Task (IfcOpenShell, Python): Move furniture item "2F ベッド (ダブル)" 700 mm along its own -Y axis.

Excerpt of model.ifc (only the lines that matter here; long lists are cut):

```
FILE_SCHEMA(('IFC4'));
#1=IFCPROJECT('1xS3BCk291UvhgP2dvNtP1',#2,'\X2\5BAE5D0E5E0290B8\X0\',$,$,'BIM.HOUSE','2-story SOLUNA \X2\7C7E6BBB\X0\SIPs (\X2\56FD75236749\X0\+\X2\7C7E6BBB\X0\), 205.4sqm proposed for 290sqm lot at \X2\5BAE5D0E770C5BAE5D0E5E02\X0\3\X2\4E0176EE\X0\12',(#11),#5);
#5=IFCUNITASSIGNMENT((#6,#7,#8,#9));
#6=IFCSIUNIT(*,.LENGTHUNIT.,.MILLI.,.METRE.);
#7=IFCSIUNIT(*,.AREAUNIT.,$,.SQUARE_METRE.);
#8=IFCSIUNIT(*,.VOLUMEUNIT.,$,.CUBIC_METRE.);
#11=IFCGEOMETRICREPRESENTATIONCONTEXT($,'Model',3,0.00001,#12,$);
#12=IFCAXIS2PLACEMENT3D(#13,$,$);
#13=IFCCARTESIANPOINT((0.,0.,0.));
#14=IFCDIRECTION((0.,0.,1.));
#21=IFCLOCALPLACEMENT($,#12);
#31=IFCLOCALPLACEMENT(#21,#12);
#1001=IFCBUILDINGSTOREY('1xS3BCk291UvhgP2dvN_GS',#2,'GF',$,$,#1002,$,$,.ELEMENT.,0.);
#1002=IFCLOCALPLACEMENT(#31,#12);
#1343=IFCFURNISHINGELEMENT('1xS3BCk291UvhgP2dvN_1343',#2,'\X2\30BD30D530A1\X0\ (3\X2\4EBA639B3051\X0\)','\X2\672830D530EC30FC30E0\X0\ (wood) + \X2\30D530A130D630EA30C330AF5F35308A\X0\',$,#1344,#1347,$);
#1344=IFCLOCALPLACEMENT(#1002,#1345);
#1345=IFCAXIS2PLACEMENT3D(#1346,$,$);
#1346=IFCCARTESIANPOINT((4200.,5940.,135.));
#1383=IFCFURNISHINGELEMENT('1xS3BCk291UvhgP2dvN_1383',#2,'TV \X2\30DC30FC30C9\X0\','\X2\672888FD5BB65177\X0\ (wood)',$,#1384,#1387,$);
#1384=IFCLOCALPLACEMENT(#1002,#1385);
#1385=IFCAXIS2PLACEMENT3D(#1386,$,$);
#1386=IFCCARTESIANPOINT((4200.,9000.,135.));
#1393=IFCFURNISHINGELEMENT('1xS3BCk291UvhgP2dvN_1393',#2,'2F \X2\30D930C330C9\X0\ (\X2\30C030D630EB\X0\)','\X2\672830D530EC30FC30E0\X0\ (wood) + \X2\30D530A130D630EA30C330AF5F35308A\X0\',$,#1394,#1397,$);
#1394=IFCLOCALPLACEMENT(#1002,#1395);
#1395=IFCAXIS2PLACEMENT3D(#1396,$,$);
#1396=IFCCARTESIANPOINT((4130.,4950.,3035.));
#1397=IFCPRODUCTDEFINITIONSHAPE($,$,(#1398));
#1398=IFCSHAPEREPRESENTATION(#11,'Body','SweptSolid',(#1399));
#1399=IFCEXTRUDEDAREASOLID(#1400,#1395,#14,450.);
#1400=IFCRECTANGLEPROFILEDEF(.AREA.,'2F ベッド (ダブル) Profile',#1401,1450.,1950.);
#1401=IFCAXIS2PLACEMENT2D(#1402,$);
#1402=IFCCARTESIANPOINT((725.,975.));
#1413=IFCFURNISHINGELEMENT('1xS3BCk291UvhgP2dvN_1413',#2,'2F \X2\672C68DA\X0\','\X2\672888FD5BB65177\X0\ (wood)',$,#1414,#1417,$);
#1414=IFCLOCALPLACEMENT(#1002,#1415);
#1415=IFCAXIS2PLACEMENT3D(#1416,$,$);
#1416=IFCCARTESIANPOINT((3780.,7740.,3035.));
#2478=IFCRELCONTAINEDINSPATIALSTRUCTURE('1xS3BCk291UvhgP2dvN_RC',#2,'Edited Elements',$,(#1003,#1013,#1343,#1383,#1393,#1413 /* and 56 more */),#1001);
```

```python
import ifcopenshell
import ifcopenshell.api.geometry
import ifcopenshell.util.placement
import ifcopenshell.util.unit

model = ifcopenshell.open("model.ifc")
unit_scale = ifcopenshell.util.unit.calculate_unit_scale(model)

item = model.by_guid("1xS3BCk291UvhgP2dvN_1393")
matrix = ifcopenshell.util.placement.get_local_placement(item.ObjectPlacement)
matrix[:3, 3] -= matrix[:3, 1] * 0.7 / unit_scale
ifcopenshell.api.geometry.edit_object_placement(model, product=item, matrix=matrix, is_si=False)

print(ifcopenshell.util.placement.get_local_placement(item.ObjectPlacement).round(3) + 0.0)

model.write("model_v2.ifc")
```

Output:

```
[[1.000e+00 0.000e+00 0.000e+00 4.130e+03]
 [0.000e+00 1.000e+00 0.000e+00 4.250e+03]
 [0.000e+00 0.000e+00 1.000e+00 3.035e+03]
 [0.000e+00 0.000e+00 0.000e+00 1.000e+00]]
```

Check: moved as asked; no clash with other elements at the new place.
